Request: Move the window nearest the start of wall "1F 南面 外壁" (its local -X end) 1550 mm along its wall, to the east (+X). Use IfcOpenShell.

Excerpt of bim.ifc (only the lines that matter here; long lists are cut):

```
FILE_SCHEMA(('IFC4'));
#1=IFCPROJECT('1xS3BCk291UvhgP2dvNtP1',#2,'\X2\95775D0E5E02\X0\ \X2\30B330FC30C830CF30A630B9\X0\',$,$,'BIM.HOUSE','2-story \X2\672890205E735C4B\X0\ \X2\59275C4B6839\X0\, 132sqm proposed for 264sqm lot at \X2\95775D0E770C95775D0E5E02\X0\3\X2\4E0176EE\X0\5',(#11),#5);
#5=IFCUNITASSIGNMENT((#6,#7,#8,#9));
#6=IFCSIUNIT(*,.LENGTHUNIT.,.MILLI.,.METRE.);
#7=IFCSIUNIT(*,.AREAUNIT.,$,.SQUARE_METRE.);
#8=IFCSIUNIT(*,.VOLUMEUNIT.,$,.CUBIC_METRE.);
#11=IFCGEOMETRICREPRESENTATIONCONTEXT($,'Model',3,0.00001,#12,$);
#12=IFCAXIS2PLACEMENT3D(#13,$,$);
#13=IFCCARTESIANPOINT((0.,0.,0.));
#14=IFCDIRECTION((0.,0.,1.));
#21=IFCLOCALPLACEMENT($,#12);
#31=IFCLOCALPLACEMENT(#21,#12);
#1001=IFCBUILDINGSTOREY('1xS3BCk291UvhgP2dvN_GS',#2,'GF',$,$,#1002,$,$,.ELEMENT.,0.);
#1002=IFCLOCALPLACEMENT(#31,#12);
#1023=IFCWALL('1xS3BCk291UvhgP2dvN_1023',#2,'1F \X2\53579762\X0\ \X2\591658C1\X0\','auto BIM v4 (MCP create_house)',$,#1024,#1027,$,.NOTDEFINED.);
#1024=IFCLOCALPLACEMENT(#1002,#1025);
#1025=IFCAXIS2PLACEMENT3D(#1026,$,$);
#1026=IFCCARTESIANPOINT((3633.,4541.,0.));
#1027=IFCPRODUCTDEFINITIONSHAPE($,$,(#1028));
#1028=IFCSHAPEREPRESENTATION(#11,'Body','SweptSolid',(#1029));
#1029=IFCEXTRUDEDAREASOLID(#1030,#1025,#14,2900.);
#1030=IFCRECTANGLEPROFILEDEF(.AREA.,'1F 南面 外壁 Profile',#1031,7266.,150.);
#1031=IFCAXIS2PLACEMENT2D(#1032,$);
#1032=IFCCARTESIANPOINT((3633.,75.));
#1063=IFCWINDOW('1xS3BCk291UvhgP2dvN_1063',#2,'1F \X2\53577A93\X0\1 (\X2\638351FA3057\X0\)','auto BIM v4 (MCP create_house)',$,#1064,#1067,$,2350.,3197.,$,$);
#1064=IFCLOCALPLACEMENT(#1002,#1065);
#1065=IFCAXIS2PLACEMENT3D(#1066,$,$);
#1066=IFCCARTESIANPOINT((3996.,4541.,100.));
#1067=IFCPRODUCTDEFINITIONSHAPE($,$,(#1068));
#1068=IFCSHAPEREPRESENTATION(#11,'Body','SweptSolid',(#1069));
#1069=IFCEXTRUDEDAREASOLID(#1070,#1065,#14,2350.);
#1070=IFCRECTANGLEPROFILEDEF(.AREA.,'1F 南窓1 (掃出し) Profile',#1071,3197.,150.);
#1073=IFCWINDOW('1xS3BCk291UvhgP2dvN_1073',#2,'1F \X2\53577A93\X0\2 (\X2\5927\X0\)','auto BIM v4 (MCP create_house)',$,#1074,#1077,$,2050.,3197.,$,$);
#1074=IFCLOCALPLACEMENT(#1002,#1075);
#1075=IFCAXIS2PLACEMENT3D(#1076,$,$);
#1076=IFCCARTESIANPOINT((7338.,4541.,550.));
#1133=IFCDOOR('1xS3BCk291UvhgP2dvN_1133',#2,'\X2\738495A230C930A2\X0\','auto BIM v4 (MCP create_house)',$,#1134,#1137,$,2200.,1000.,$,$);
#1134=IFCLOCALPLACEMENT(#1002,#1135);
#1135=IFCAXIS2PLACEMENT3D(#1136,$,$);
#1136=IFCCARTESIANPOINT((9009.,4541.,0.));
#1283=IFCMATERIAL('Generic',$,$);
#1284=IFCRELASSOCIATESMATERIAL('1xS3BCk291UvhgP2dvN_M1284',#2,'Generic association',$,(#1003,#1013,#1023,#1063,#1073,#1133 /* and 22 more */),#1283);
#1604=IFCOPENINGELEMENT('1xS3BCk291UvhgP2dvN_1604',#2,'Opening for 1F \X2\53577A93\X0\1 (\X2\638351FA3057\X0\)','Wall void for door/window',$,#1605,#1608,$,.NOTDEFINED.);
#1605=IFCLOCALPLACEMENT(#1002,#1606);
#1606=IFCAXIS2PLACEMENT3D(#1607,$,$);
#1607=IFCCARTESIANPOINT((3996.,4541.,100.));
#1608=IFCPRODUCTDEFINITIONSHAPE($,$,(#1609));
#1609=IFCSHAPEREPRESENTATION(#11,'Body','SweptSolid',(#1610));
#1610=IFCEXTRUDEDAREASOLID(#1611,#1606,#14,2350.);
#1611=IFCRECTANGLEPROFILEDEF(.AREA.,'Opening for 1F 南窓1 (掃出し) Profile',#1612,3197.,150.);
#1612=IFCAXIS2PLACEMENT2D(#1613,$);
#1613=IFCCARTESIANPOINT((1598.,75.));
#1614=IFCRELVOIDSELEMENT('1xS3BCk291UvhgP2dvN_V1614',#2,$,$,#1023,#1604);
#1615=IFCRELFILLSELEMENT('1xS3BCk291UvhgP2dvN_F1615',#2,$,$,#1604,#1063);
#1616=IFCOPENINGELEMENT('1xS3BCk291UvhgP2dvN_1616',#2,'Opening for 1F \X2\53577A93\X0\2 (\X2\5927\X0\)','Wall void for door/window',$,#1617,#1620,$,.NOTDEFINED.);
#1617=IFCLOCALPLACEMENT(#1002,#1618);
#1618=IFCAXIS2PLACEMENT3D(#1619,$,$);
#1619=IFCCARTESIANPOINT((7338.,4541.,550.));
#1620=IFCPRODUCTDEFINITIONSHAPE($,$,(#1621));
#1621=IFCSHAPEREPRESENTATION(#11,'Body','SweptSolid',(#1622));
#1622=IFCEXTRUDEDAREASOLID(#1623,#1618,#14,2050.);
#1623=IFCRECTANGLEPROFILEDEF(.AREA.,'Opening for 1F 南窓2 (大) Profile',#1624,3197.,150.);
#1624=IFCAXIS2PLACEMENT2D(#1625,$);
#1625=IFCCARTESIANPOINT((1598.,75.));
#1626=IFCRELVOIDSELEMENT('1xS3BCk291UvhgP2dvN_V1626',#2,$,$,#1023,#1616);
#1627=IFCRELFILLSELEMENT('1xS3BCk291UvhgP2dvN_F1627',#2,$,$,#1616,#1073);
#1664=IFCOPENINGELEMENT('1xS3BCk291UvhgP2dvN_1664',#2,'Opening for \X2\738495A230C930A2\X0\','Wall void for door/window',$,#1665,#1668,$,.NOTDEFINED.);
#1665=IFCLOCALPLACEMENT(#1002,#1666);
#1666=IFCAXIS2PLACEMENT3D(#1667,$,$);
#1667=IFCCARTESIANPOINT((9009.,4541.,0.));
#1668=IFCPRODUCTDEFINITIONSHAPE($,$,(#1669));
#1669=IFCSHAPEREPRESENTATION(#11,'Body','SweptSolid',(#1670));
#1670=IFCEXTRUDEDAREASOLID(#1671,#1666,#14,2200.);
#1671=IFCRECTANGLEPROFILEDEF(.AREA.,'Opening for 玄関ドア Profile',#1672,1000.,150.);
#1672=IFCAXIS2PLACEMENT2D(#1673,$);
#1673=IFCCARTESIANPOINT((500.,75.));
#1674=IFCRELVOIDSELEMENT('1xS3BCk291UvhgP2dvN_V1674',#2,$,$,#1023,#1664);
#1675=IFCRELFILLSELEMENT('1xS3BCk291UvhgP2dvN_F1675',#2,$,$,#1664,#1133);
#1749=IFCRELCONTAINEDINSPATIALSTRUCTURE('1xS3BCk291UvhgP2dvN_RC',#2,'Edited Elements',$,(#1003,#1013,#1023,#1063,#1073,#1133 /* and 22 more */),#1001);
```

```python
import ifcopenshell
import ifcopenshell.api.geometry
import ifcopenshell.util.placement

model = ifcopenshell.open("bim.ifc")

window = model.by_id(1063)
opening = window.FillsVoids[0].RelatingOpeningElement
wall = opening.VoidsElements[0].RelatingBuildingElement

wall_matrix = ifcopenshell.util.placement.get_local_placement(wall.ObjectPlacement)
shift = wall_matrix[:3, 0] * 1550.0
before = ifcopenshell.util.placement.get_local_placement(window.ObjectPlacement)[:3, 3].copy()

# The window is not placed relative to its opening, so move both.
for product in (opening, window):
    matrix = ifcopenshell.util.placement.get_local_placement(product.ObjectPlacement)
    matrix[:3, 3] += shift
    ifcopenshell.api.geometry.edit_object_placement(model, product=product, matrix=matrix, is_si=False)

after = ifcopenshell.util.placement.get_local_placement(window.ObjectPlacement)[:3, 3]
print("window moved by", (after - before).round(3) + 0.0)

model.write("bim-out.ifc")
```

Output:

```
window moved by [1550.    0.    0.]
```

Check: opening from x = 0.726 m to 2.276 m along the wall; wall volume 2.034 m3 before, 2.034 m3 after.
